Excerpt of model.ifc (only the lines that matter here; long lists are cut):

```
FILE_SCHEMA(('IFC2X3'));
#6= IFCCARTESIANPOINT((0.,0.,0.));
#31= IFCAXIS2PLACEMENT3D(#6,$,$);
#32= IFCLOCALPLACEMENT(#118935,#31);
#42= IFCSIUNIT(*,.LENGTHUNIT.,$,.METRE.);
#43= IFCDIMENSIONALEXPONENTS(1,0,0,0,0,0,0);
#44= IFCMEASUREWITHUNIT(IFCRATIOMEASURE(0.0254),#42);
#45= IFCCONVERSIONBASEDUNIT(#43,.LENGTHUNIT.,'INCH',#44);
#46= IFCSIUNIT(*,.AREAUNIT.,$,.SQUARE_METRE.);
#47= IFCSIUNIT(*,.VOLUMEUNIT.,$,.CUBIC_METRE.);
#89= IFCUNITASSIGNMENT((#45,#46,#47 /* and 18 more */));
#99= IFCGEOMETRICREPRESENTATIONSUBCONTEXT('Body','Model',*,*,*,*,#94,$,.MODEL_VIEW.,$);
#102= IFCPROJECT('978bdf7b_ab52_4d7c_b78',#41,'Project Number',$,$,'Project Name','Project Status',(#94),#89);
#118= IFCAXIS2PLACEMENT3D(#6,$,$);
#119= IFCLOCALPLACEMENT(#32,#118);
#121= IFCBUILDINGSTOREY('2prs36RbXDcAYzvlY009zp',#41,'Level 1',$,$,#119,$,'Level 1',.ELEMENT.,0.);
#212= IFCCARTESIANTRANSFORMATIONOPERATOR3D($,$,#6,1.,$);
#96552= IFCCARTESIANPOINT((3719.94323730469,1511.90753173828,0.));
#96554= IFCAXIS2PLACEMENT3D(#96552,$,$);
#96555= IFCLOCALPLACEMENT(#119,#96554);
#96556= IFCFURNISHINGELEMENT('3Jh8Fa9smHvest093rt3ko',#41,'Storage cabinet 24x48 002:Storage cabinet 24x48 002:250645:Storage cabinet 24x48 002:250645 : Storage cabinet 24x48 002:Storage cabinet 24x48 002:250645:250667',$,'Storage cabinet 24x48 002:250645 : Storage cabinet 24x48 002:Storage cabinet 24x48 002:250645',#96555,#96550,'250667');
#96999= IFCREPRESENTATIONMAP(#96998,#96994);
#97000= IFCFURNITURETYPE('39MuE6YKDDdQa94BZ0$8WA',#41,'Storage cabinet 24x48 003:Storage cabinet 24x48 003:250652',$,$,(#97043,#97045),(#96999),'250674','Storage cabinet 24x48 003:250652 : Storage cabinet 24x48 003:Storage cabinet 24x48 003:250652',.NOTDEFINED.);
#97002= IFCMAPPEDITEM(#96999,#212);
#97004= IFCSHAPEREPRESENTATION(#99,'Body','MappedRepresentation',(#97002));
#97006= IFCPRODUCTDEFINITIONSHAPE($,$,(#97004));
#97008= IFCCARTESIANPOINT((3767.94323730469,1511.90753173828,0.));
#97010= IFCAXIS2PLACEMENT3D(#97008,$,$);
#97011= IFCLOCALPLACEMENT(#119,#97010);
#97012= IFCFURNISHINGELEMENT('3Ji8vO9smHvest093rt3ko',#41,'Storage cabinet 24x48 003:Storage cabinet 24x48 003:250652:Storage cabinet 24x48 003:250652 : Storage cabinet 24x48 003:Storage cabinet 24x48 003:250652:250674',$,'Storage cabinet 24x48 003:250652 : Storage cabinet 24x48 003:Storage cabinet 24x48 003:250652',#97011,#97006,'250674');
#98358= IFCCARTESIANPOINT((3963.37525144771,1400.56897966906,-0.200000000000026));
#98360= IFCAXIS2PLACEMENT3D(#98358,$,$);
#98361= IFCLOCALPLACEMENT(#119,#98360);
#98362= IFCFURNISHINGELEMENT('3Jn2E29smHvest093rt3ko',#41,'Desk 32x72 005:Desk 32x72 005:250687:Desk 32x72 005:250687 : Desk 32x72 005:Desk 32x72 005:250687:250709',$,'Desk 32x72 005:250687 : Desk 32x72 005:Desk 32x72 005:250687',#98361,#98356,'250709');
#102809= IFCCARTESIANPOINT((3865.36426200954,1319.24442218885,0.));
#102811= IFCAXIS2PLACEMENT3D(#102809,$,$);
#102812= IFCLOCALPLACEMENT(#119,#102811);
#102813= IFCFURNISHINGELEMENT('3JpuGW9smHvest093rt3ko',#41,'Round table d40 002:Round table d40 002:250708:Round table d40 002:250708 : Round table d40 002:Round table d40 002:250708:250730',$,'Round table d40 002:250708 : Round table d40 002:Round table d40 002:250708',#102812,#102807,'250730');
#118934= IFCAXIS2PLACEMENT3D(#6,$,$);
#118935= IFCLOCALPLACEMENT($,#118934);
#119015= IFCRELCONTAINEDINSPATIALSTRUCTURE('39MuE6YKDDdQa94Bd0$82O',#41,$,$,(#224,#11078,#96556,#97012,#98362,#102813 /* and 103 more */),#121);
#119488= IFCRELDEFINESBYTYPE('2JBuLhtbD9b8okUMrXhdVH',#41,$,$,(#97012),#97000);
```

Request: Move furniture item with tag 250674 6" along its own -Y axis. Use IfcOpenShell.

```python
import ifcopenshell
import ifcopenshell.api.geometry
import ifcopenshell.util.placement
import ifcopenshell.util.unit

model = ifcopenshell.open("model.ifc")
unit_scale = ifcopenshell.util.unit.calculate_unit_scale(model)

item = model.by_guid("3Ji8vO9smHvest093rt3ko")
matrix = ifcopenshell.util.placement.get_local_placement(item.ObjectPlacement)
matrix[:3, 3] -= matrix[:3, 1] * 6 * 0.0254 / unit_scale
ifcopenshell.api.geometry.edit_object_placement(model, product=item, matrix=matrix, is_si=False)

print(ifcopenshell.util.placement.get_local_placement(item.ObjectPlacement).round(3) + 0.0)

model.write("model_updated.ifc")
```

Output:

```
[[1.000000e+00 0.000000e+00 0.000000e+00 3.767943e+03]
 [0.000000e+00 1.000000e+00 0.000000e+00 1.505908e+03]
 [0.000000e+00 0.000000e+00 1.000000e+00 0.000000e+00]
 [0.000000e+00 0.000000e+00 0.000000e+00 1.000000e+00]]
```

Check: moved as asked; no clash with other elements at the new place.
